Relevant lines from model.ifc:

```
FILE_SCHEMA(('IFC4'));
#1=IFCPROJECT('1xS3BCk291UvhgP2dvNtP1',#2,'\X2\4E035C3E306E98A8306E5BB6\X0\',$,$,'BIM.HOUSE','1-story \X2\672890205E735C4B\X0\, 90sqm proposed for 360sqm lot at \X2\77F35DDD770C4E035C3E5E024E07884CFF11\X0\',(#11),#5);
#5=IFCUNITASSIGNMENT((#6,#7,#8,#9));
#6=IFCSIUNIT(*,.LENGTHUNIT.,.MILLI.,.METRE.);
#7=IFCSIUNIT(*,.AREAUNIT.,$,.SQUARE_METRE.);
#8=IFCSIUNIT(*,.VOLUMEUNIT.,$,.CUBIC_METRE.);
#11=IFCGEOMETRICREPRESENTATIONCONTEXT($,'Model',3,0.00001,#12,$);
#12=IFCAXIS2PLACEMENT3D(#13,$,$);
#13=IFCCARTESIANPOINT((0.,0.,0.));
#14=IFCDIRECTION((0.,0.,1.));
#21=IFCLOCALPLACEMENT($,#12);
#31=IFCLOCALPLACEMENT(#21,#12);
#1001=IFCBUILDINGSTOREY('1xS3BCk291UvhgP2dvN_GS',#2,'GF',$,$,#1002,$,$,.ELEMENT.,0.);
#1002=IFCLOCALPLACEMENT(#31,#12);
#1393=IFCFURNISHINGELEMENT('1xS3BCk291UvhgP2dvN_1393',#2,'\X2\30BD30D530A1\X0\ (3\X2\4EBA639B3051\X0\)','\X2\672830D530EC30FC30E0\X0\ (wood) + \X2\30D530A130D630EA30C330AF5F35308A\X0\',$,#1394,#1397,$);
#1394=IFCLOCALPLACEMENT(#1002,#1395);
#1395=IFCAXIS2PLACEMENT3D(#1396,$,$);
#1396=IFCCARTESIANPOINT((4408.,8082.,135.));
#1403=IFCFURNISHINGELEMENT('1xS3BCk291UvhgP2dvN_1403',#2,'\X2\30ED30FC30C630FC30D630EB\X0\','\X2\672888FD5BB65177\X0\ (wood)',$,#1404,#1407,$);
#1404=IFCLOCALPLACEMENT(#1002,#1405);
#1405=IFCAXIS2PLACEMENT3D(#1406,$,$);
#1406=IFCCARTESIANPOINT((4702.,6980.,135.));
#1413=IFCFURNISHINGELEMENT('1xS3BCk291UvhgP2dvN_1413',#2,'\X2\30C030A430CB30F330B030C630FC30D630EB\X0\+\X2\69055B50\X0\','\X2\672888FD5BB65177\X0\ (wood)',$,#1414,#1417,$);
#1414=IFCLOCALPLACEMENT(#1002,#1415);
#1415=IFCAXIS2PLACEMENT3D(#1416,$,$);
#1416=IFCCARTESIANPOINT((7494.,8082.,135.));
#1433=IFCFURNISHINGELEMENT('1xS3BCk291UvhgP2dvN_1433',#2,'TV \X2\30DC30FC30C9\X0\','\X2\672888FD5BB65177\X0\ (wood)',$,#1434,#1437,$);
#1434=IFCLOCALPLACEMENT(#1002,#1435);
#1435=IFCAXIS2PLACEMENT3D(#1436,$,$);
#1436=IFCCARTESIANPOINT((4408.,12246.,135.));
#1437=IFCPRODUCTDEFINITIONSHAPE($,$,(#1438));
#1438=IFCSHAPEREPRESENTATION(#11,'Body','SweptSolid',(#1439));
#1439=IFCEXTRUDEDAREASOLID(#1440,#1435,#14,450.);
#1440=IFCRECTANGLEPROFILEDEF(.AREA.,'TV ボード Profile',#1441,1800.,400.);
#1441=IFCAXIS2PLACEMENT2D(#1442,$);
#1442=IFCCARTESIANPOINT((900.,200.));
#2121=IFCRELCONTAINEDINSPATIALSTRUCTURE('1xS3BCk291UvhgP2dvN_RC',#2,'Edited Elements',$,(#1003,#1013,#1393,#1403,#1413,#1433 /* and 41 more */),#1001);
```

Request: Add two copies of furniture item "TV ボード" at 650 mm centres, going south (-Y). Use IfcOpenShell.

```python
import numpy as np
import ifcopenshell
import ifcopenshell.api.geometry
import ifcopenshell.api.root
import ifcopenshell.util.element
import ifcopenshell.util.placement
import ifcopenshell.util.unit

model = ifcopenshell.open("model.ifc")
unit_scale = ifcopenshell.util.unit.calculate_unit_scale(model)


def reuse_history(source, copy):
    """copy_class also copies each property set's owner history, people and application; keep the originals."""
    for rel in copy.IsDefinedBy:
        if rel.is_a("IfcRelDefinesByProperties") and (history := rel.RelatingPropertyDefinition.OwnerHistory):
            rel.RelatingPropertyDefinition.OwnerHistory = source.OwnerHistory
            ifcopenshell.util.element.remove_deep2(model, history)


source = model.by_guid("1xS3BCk291UvhgP2dvN_1433")
base = ifcopenshell.util.placement.get_local_placement(source.ObjectPlacement)
step = np.array([0.0, -1.0, 0.0]) * 0.65 / unit_scale

for i in range(1, 3):
    copy = ifcopenshell.api.root.copy_class(model, product=source)
    copy.Representation = ifcopenshell.util.element.copy_deep(
        model, source.Representation, exclude=["IfcGeometricRepresentationContext", "IfcRepresentationMap"]
    )
    reuse_history(source, copy)
    matrix = base.copy()
    matrix[:3, 3] += i * step
    print("added at", matrix[:3, 3].round(3) + 0.0)
    ifcopenshell.api.geometry.edit_object_placement(model, product=copy, matrix=matrix, is_si=False)

model.write("model_updated.ifc")
```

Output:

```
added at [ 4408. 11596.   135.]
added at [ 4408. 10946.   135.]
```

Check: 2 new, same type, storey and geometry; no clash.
